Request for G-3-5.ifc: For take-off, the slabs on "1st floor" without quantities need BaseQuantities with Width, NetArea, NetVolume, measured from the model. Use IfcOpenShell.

First a look at what the model holds.

```python
import ifcopenshell
import ifcopenshell.util.element
import ifcopenshell.util.unit

model = ifcopenshell.open("G-3-5.ifc")
print(model.schema)
for unit_type in ("LENGTHUNIT", "AREAUNIT", "VOLUMEUNIT"):
    print(unit_type, ifcopenshell.util.unit.calculate_unit_scale(model, unit_type))
storey = next(s for s in model.by_type("IfcBuildingStorey") if s.Name == "1st floor")
slabs = [e for e in ifcopenshell.util.element.get_decomposition(storey) if e.is_a("IfcSlab")]
for e in sorted(slabs, key=lambda e: e.id()):
    print(e.id(), e.is_a(), e.Name, list(ifcopenshell.util.element.get_psets(e, qtos_only=True)), sep=" | ")
```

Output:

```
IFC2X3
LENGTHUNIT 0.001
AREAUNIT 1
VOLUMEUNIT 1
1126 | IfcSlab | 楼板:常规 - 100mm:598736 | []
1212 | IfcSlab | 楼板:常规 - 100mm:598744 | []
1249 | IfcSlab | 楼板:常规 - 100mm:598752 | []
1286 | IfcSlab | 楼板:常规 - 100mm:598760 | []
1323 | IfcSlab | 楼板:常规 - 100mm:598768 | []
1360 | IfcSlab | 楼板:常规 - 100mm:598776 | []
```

```python
import ifcopenshell
import ifcopenshell.api.pset
import ifcopenshell.geom
import ifcopenshell.util.element
import ifcopenshell.util.shape
import ifcopenshell.util.unit

model = ifcopenshell.open("G-3-5.ifc")
unit_scale = ifcopenshell.util.unit.calculate_unit_scale(model)
area_scale = ifcopenshell.util.unit.calculate_unit_scale(model, "AREAUNIT")
volume_scale = ifcopenshell.util.unit.calculate_unit_scale(model, "VOLUMEUNIT")
settings = ifcopenshell.geom.settings()

storey = next(s for s in model.by_type("IfcBuildingStorey") if s.Name == "1st floor")
slabs = [e for e in ifcopenshell.util.element.get_decomposition(storey) if e.is_a("IfcSlab")]

for e in sorted(slabs, key=lambda e: e.id()):
    if ifcopenshell.util.element.get_psets(e, qtos_only=True, should_inherit=False):
        continue
    # Geometry comes back in metres, in the element's own axes.
    shape = ifcopenshell.geom.create_shape(settings, e)
    values = {
        "Width": ifcopenshell.util.shape.get_z(shape.geometry) / unit_scale,
        "NetArea": ifcopenshell.util.shape.get_footprint_area(shape.geometry) / area_scale,
        "NetVolume": ifcopenshell.util.shape.get_volume(shape.geometry) / volume_scale,
    }
    qto = ifcopenshell.api.pset.add_qto(model, product=e, name="BaseQuantities")
    ifcopenshell.api.pset.edit_qto(model, qto=qto, properties=values)
    print(e.id(), {k: round(v, 3) for k, v in values.items()})

model.write("G-3-5-out.ifc")
```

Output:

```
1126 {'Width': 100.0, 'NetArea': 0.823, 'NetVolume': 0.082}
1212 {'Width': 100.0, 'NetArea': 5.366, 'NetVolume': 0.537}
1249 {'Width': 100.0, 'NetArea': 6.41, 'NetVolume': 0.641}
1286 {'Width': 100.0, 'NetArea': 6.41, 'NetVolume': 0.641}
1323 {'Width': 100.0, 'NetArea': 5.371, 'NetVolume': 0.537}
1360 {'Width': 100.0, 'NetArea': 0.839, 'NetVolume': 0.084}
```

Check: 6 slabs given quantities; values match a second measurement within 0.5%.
